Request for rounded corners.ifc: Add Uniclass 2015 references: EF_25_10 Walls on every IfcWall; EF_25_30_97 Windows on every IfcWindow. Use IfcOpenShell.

First a look at what the model holds.

```python
import ifcopenshell

model = ifcopenshell.open("rounded corners.ifc")
print(model.schema)
print("classifications:", [c.Name for c in model.by_type("IfcClassification")])
for ifc_class in ("IfcDoor", "IfcRoof", "IfcStair", "IfcWall", "IfcWindow"):
    print(ifc_class, len(model.by_type(ifc_class)))
```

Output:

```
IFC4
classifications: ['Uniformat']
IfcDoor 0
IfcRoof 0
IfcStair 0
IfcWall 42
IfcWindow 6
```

```python
import ifcopenshell
import ifcopenshell.api.classification

model = ifcopenshell.open("rounded corners.ifc")

system = ifcopenshell.api.classification.add_classification(model, classification="Uniclass 2015")

codes = {
    "IfcWall": ("EF_25_10", "Walls"),
    "IfcWindow": ("EF_25_30_97", "Windows"),
}
for ifc_class, (code, name) in codes.items():
    products = model.by_type(ifc_class)
    ifcopenshell.api.classification.add_reference(
        model, products=products, classification=system, identification=code, name=name
    )
    print(code, len(products))

model.write("rounded corners_edited.ifc")
```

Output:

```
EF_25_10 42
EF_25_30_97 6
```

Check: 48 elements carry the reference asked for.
